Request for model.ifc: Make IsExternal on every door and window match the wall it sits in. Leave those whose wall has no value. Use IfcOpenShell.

First a look at what the model holds.

```python
import ifcopenshell
import ifcopenshell.util.element

model = ifcopenshell.open("model.ifc")
print(model.schema)
seen = {}
for e in model.by_type("IfcDoor") + model.by_type("IfcWindow"):
    if not e.FillsVoids:
        continue
    host = e.FillsVoids[0].RelatingOpeningElement.VoidsElements[0].RelatingBuildingElement
    own = ifcopenshell.util.element.get_pset(e, f"Pset_{e.is_a()[3:].removesuffix('StandardCase')}Common", "IsExternal")
    wall = ifcopenshell.util.element.get_pset(host, "Pset_WallCommon", "IsExternal")
    seen[e.is_a(), own, wall] = seen.get((e.is_a(), own, wall), 0) + 1
for (cls, own, wall), count in sorted(seen.items(), key=str):
    print(count, cls, "IsExternal:", own, "| host wall:", wall)
```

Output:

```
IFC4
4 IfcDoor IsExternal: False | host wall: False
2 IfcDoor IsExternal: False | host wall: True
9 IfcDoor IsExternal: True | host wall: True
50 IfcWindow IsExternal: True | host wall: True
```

```python
import ifcopenshell
import ifcopenshell.api.pset
import ifcopenshell.util.element

model = ifcopenshell.open("model.ifc")

count = 0
for ifc_class, pset_name in (("IfcDoor", "Pset_DoorCommon"), ("IfcWindow", "Pset_WindowCommon")):
    for e in model.by_type(ifc_class):
        if not e.FillsVoids:
            continue
        host = e.FillsVoids[0].RelatingOpeningElement.VoidsElements[0].RelatingBuildingElement
        external = ifcopenshell.util.element.get_pset(host, "Pset_WallCommon", "IsExternal")
        if external is None or ifcopenshell.util.element.get_pset(e, pset_name, "IsExternal") == external:
            continue
        pset = ifcopenshell.api.pset.add_pset(model, product=e, name=pset_name)
        ifcopenshell.api.pset.edit_pset(model, pset=pset, properties={"IsExternal": external})
        count += 1

print(count, "updated")

model.write("model_rev.ifc")
```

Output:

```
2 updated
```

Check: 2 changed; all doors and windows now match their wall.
